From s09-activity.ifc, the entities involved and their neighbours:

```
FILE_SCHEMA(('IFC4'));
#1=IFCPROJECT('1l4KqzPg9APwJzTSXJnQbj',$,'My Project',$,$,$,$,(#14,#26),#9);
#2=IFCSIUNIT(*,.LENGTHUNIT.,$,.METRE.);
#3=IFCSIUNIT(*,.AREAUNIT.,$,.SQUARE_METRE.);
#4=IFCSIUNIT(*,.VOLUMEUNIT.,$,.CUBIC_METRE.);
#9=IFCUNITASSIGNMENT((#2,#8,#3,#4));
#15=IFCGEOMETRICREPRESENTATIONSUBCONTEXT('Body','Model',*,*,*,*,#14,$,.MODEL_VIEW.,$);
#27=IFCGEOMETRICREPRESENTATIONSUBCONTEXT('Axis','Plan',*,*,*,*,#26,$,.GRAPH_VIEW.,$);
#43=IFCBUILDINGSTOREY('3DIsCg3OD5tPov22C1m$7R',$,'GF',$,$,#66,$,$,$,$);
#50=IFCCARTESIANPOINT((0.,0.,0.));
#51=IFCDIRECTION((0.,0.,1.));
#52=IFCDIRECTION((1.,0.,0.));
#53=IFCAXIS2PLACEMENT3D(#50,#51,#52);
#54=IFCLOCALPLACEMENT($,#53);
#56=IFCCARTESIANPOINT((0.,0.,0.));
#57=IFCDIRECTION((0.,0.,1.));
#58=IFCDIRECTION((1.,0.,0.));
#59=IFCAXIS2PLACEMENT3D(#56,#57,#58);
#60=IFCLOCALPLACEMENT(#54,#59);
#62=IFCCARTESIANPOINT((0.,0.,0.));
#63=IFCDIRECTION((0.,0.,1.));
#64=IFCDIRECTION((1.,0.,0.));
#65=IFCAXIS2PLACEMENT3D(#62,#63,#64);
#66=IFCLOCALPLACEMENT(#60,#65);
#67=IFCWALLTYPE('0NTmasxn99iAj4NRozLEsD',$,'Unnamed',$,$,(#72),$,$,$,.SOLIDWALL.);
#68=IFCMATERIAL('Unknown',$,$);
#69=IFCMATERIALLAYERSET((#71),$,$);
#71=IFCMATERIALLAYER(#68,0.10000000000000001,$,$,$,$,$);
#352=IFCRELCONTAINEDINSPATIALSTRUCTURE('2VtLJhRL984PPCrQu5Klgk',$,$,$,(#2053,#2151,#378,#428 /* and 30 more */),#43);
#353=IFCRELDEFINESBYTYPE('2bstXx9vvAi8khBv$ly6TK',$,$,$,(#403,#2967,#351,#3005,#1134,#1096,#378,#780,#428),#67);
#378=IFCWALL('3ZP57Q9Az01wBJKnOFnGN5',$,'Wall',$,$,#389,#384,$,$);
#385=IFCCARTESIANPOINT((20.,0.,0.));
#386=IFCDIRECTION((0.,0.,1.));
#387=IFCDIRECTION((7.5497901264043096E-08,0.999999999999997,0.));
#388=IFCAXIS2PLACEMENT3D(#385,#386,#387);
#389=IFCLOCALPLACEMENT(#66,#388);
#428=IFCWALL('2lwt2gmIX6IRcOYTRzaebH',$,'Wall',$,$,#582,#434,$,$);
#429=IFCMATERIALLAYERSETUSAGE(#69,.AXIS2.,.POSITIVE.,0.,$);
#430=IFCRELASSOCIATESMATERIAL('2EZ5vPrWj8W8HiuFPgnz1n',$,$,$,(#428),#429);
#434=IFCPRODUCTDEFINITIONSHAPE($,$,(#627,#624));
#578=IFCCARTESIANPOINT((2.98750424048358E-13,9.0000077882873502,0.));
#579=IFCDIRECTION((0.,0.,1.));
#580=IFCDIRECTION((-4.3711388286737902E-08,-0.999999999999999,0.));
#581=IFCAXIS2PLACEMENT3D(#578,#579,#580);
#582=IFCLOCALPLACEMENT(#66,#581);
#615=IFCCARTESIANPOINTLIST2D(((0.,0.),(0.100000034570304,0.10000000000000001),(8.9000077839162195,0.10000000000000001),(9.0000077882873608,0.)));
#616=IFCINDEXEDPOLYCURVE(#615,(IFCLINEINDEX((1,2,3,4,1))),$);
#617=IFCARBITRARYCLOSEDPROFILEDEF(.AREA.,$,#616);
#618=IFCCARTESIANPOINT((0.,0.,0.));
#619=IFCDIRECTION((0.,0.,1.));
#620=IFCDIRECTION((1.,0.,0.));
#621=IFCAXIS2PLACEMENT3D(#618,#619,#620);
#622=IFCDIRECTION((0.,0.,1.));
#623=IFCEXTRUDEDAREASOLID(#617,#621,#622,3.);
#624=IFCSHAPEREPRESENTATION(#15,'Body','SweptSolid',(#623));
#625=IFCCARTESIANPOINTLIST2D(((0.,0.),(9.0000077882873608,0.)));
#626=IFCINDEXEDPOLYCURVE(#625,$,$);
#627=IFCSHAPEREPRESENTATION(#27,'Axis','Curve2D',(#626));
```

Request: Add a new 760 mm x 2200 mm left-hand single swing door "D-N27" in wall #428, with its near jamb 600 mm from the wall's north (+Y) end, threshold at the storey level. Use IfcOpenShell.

```python
import numpy as np
import ifcopenshell
import ifcopenshell.api.feature
import ifcopenshell.api.geometry
import ifcopenshell.api.root
import ifcopenshell.api.spatial
import ifcopenshell.geom
import ifcopenshell.util.element
import ifcopenshell.util.placement
import ifcopenshell.util.representation
import ifcopenshell.util.shape
import ifcopenshell.util.unit

model = ifcopenshell.open("s09-activity.ifc")
unit_scale = ifcopenshell.util.unit.calculate_unit_scale(model)
settings = ifcopenshell.geom.settings()


def volume(element):
    """Net volume in cubic metres, openings subtracted."""
    shape = ifcopenshell.geom.create_shape(settings, element)
    return ifcopenshell.util.shape.get_volume(shape.geometry)


wall = model.by_guid("2lwt2gmIX6IRcOYTRzaebH")
storey = ifcopenshell.util.element.get_container(wall, ifc_class="IfcBuildingStorey")
context = ifcopenshell.util.representation.get_context(model, "Model", "Body", "MODEL_VIEW")
before = volume(wall)

width, height, from_end, sill = 0.76, 2.2, 0.6, 0.0  # metres

# The wall runs along its own X axis, and the end named is its -X end.
wall_shape = ifcopenshell.geom.create_shape(settings, wall)
x, y, z = ifcopenshell.util.shape.get_vertices(wall_shape.geometry).T
start = x.min() + from_end
face, thickness = float(y.min()), float(y.max() - y.min())
wall_matrix = ifcopenshell.util.placement.get_local_placement(wall.ObjectPlacement)
level = ifcopenshell.util.placement.get_local_placement(storey.ObjectPlacement)[2, 3]


def in_wall(x, y):
    """Placement at x, y metres in the wall's axes, at sill height."""
    matrix = wall_matrix.copy()
    matrix[:, 3] = wall_matrix @ np.array([x / unit_scale, y / unit_scale, 0.0, 1.0])
    matrix[2, 3] = level + sill / unit_scale
    return matrix


# Opening: a box that overshoots both wall faces by 50 mm.
opening = ifcopenshell.api.root.create_entity(model, ifc_class="IfcOpeningElement", predefined_type="OPENING")
box = ifcopenshell.api.geometry.add_wall_representation(
    model, context=context, length=width, height=height, thickness=thickness + 0.1
)
ifcopenshell.api.geometry.assign_representation(model, product=opening, representation=box)
ifcopenshell.api.geometry.edit_object_placement(model, product=opening, matrix=in_wall(start, face - 0.05), is_si=False)
ifcopenshell.api.feature.add_feature(model, feature=opening, element=wall)

door = ifcopenshell.api.root.create_entity(model, ifc_class="IfcDoor", name="D-N27", predefined_type="DOOR")
door.OverallWidth, door.OverallHeight = width / unit_scale, height / unit_scale
door.OperationType = "SINGLE_SWING_LEFT"
body = ifcopenshell.api.geometry.add_door_representation(
    model,
    context=context,
    overall_width=door.OverallWidth,
    overall_height=door.OverallHeight,
    operation_type="SINGLE_SWING_LEFT",
    lining_properties={"LiningDepth": thickness / unit_scale, "ThresholdDepth": thickness / unit_scale},
)
ifcopenshell.api.geometry.assign_representation(model, product=door, representation=body)
ifcopenshell.api.spatial.assign_container(model, products=[door], relating_structure=storey)
ifcopenshell.api.feature.add_filling(model, opening=opening, element=door)

# The lining spans the wall, so the door starts at the wall face.
ifcopenshell.api.geometry.edit_object_placement(model, product=door, matrix=in_wall(start, face), is_si=False)

after = volume(wall)

print(f"wall volume {before:.3f} -> {after:.3f} m3")

model.write("s09-activity_updated.ifc")
```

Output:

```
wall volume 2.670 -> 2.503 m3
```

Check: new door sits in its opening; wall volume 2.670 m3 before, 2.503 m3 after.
